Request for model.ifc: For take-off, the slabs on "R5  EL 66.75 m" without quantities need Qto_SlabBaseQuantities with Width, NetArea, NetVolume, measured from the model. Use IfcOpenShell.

First a look at what the model holds.

```python
import ifcopenshell
import ifcopenshell.util.element
import ifcopenshell.util.unit

model = ifcopenshell.open("model.ifc")
print(model.schema)
for unit_type in ("LENGTHUNIT", "AREAUNIT", "VOLUMEUNIT"):
    print(unit_type, ifcopenshell.util.unit.calculate_unit_scale(model, unit_type))
storey = next(s for s in model.by_type("IfcBuildingStorey") if s.Name == "R5  EL 66.75 m")
slabs = [e for e in ifcopenshell.util.element.get_decomposition(storey) if e.is_a("IfcSlab")]
for e in sorted(slabs, key=lambda e: e.id()):
    print(e.id(), e.is_a(), e.Name, list(ifcopenshell.util.element.get_psets(e, qtos_only=True)), sep=" | ")
```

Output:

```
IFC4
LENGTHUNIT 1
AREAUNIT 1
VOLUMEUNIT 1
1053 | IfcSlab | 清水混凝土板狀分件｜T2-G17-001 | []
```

```python
import ifcopenshell
import ifcopenshell.api.pset
import ifcopenshell.geom
import ifcopenshell.util.element
import ifcopenshell.util.shape
import ifcopenshell.util.unit

model = ifcopenshell.open("model.ifc")
unit_scale = ifcopenshell.util.unit.calculate_unit_scale(model)
area_scale = ifcopenshell.util.unit.calculate_unit_scale(model, "AREAUNIT")
volume_scale = ifcopenshell.util.unit.calculate_unit_scale(model, "VOLUMEUNIT")
settings = ifcopenshell.geom.settings()

storey = next(s for s in model.by_type("IfcBuildingStorey") if s.Name == "R5  EL 66.75 m")
slabs = [e for e in ifcopenshell.util.element.get_decomposition(storey) if e.is_a("IfcSlab")]

for e in sorted(slabs, key=lambda e: e.id()):
    if ifcopenshell.util.element.get_psets(e, qtos_only=True, should_inherit=False):
        continue
    # Geometry comes back in metres, in the element's own axes.
    shape = ifcopenshell.geom.create_shape(settings, e)
    values = {
        "Width": ifcopenshell.util.shape.get_z(shape.geometry) / unit_scale,
        "NetArea": ifcopenshell.util.shape.get_footprint_area(shape.geometry) / area_scale,
        "NetVolume": ifcopenshell.util.shape.get_volume(shape.geometry) / volume_scale,
    }
    qto = ifcopenshell.api.pset.add_qto(model, product=e, name="Qto_SlabBaseQuantities")
    ifcopenshell.api.pset.edit_qto(model, qto=qto, properties=values)
    print(e.id(), {k: round(v, 3) for k, v in values.items()})

model.write("model_rev.ifc")
```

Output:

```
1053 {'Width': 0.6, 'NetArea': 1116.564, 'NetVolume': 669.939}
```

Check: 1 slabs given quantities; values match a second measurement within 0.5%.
